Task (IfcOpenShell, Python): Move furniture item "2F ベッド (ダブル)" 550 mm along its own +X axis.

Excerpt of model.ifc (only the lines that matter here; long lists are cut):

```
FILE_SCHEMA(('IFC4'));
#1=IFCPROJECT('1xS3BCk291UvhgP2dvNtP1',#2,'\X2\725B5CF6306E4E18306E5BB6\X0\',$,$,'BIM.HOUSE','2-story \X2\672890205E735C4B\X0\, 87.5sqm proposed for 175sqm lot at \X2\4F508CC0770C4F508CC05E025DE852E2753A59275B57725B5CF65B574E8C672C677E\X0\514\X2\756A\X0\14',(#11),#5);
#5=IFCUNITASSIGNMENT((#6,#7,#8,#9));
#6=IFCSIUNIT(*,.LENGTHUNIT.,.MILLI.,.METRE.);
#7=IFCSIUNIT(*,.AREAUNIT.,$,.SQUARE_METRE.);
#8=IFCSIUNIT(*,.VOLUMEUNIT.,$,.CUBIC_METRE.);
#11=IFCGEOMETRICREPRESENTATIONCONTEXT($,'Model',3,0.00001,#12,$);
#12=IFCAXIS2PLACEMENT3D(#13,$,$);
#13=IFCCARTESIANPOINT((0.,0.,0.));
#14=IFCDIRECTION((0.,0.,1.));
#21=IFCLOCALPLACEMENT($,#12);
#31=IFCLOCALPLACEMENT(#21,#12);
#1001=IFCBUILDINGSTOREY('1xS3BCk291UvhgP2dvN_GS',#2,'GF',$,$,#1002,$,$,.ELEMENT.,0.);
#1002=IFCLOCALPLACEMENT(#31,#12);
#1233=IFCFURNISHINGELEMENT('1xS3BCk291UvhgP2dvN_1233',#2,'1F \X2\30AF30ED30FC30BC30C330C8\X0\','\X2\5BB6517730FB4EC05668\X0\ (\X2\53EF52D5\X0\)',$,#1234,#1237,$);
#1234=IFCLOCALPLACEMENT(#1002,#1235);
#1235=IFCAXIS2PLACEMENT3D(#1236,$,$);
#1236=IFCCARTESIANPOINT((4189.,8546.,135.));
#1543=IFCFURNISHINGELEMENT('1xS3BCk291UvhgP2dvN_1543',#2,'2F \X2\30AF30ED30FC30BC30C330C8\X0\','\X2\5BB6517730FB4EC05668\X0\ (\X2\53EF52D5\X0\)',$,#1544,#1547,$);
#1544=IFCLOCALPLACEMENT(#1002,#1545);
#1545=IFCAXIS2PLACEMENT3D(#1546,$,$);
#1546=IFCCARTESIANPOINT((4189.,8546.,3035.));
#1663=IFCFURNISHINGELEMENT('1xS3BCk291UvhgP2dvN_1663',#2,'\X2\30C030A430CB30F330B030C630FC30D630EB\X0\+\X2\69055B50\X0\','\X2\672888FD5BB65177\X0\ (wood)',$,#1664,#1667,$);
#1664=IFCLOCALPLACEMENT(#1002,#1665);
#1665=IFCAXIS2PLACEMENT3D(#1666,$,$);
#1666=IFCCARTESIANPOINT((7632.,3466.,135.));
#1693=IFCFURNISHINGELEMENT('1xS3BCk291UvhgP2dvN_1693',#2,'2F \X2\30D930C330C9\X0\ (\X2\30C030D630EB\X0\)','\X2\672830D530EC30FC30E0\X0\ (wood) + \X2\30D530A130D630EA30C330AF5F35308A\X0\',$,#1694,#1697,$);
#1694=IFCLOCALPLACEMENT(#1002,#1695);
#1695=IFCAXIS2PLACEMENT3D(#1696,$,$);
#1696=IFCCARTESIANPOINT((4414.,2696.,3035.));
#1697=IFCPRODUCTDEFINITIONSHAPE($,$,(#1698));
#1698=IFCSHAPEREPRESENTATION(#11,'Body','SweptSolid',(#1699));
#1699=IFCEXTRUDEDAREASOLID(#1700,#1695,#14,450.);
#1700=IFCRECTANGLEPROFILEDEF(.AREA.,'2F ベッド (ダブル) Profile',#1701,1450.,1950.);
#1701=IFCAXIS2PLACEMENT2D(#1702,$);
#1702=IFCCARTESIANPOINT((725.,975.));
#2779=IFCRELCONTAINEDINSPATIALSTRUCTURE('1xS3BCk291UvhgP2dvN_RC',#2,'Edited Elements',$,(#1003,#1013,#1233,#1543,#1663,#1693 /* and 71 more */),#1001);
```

```python
import ifcopenshell
import ifcopenshell.api.geometry
import ifcopenshell.util.placement
import ifcopenshell.util.unit

model = ifcopenshell.open("model.ifc")
unit_scale = ifcopenshell.util.unit.calculate_unit_scale(model)

item = model.by_guid("1xS3BCk291UvhgP2dvN_1693")
matrix = ifcopenshell.util.placement.get_local_placement(item.ObjectPlacement)
matrix[:3, 3] += matrix[:3, 0] * 0.55 / unit_scale
ifcopenshell.api.geometry.edit_object_placement(model, product=item, matrix=matrix, is_si=False)

print(ifcopenshell.util.placement.get_local_placement(item.ObjectPlacement).round(3) + 0.0)

model.write("model_rev.ifc")
```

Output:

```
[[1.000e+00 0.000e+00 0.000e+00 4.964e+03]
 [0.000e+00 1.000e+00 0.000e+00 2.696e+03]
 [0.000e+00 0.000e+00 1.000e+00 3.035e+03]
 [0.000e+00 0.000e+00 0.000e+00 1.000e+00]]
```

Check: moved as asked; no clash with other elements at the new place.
